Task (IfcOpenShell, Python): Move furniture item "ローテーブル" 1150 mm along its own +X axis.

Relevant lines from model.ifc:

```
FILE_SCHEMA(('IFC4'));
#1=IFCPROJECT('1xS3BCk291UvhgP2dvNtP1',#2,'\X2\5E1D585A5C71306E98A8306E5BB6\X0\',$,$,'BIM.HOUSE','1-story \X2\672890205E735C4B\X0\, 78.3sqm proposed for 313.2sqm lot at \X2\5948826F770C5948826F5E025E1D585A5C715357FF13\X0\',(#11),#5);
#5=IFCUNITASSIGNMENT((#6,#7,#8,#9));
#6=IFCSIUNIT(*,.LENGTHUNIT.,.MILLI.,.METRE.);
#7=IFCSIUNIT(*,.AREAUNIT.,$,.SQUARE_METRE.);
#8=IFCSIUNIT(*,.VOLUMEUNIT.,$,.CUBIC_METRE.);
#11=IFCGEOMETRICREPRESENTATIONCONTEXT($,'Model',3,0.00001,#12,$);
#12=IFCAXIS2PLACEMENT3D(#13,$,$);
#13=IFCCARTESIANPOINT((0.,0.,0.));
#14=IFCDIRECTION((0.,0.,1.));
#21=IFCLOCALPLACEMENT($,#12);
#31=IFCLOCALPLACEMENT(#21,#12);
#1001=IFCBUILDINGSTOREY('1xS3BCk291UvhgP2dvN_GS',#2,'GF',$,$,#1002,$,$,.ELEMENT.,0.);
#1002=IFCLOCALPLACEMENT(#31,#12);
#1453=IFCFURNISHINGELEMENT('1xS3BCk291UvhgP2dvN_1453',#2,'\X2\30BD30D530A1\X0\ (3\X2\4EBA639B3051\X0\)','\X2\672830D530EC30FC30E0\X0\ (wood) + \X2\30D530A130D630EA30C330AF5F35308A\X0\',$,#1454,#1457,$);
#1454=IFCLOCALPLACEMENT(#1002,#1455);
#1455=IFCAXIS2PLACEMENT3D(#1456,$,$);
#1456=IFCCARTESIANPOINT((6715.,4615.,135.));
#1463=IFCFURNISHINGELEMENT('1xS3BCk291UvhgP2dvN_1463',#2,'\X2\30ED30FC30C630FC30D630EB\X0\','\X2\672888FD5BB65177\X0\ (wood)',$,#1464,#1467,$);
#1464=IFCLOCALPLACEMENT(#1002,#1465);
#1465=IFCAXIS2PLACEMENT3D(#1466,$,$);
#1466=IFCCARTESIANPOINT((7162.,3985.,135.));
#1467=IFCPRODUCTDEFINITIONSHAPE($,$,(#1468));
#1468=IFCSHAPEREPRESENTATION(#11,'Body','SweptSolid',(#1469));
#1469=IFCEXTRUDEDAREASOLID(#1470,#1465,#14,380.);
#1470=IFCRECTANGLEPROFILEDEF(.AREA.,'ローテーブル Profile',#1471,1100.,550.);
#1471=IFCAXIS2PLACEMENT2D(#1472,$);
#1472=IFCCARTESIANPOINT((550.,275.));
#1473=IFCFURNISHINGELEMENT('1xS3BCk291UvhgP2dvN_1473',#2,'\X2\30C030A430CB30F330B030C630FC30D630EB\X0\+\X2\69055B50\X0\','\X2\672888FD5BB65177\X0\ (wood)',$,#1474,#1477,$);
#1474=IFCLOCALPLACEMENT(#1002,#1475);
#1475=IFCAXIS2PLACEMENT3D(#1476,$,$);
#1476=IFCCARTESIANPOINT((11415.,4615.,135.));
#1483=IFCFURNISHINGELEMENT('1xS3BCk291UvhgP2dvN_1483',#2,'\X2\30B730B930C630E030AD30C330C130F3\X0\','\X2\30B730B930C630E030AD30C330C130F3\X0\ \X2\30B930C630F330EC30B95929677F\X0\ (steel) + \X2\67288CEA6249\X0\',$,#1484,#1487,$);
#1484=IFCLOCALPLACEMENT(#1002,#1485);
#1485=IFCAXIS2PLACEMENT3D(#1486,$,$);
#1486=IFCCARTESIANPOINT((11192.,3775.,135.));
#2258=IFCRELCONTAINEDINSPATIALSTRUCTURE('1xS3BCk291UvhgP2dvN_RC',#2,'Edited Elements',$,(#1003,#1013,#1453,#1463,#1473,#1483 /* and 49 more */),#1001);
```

```python
import ifcopenshell
import ifcopenshell.api.geometry
import ifcopenshell.util.placement

model = ifcopenshell.open("model.ifc")

item = model.by_guid("1xS3BCk291UvhgP2dvN_1463")
matrix = ifcopenshell.util.placement.get_local_placement(item.ObjectPlacement)
matrix[:3, 3] += matrix[:3, 0] * 1150.0
ifcopenshell.api.geometry.edit_object_placement(model, product=item, matrix=matrix, is_si=False)

print(ifcopenshell.util.placement.get_local_placement(item.ObjectPlacement).round(3) + 0.0)

model.write("model_updated.ifc")
```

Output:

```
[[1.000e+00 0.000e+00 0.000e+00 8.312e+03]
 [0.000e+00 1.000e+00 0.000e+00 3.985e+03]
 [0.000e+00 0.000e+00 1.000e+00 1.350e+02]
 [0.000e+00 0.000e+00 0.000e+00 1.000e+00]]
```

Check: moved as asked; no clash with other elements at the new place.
